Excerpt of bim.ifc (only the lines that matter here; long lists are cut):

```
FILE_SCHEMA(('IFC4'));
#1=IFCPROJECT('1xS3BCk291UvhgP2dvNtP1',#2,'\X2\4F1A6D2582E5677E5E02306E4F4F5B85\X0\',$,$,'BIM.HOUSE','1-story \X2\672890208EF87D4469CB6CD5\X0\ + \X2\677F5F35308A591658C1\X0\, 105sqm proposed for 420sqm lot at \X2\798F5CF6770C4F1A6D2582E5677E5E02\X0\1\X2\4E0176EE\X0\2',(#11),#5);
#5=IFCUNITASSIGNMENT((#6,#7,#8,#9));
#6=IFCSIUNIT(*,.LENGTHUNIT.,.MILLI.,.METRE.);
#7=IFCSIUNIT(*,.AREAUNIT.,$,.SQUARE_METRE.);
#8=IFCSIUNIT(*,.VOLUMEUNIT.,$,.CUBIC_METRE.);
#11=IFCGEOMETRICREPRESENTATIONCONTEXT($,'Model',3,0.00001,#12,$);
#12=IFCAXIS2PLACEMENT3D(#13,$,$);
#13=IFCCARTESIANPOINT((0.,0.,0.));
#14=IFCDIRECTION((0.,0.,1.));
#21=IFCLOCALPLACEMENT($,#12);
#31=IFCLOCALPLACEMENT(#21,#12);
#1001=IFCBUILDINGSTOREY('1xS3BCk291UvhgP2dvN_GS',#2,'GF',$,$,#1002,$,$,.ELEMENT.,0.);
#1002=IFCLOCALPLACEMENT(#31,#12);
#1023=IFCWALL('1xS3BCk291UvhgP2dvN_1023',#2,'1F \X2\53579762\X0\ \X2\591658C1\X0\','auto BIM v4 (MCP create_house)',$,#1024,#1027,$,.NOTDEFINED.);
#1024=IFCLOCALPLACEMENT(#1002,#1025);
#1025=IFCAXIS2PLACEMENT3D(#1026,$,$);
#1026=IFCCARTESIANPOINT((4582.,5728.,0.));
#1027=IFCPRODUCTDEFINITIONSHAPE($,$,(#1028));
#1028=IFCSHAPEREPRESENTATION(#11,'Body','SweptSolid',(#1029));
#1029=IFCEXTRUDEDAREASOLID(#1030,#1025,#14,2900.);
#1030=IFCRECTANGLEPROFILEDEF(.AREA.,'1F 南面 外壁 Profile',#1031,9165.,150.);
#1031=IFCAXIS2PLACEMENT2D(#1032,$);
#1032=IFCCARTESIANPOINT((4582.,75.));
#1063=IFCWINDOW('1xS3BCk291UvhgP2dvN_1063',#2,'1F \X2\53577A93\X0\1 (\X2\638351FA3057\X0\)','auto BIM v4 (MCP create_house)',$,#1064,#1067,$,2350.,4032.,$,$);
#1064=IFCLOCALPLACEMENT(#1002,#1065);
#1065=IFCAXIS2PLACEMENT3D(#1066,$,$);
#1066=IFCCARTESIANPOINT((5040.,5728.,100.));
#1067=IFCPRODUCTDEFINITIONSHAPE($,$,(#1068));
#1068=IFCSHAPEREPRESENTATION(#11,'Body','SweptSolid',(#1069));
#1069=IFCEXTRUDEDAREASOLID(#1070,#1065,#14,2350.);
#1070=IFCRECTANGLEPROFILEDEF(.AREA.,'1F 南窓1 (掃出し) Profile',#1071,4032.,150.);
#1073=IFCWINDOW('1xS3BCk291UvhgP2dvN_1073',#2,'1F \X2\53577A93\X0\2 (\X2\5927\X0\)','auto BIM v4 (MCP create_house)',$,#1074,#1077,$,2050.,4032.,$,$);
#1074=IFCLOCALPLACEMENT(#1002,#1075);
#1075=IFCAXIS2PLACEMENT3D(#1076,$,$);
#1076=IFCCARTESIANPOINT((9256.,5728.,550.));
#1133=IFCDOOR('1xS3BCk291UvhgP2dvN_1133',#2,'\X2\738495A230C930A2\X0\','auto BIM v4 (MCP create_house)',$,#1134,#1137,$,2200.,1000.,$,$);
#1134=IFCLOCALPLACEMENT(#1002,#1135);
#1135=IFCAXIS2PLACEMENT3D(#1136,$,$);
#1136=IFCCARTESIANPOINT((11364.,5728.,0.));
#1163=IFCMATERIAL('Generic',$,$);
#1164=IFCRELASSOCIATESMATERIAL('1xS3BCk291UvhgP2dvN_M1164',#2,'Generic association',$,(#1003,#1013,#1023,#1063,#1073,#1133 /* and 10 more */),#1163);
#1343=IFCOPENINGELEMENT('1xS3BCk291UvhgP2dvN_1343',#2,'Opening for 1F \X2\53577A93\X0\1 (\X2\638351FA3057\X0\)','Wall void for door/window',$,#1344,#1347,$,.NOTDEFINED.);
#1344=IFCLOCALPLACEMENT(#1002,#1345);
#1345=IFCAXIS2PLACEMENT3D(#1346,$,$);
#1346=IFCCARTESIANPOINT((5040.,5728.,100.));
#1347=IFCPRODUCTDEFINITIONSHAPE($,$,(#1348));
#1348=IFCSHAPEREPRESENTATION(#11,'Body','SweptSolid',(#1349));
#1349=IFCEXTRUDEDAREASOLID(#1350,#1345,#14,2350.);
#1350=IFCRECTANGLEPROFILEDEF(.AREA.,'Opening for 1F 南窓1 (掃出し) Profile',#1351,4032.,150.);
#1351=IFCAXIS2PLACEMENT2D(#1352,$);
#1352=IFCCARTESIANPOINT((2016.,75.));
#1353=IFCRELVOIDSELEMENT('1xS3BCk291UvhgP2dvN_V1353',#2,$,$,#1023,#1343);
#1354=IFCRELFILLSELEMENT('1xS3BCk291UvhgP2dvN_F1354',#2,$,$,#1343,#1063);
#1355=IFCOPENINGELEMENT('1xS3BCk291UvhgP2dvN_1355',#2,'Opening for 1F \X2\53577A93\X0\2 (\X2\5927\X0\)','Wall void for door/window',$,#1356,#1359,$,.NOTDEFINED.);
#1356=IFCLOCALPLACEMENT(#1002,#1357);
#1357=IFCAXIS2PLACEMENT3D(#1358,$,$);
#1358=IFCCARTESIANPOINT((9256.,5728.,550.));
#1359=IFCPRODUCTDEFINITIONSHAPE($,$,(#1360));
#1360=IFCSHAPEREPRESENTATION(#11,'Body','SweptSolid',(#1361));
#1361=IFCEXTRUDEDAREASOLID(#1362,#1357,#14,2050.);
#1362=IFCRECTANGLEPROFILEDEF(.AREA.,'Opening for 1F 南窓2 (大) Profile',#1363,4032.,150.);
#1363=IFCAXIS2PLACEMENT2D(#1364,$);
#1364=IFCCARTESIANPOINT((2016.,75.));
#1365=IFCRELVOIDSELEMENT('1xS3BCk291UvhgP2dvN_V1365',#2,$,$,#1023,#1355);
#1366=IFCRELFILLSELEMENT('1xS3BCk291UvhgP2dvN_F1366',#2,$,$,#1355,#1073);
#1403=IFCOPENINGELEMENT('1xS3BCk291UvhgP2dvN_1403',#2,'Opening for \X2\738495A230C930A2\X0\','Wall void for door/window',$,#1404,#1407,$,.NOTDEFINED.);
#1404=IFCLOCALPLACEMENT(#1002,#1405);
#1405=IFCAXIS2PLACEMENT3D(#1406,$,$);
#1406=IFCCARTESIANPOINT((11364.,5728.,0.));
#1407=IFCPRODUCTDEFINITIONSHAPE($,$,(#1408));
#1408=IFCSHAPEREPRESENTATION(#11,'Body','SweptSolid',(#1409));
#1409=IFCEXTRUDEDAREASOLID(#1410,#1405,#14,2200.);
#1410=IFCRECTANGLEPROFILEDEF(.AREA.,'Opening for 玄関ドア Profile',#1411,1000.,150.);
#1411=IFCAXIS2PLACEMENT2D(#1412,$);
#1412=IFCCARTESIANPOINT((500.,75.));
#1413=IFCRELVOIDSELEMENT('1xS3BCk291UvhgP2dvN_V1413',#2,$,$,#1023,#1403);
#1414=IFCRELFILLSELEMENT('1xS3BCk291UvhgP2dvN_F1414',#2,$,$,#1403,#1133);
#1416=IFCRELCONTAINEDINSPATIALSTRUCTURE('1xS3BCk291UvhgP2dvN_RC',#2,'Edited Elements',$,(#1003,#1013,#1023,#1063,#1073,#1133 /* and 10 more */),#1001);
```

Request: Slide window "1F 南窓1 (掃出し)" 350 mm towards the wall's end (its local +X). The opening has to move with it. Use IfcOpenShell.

```python
import ifcopenshell
import ifcopenshell.api.geometry
import ifcopenshell.util.placement
import ifcopenshell.util.unit

model = ifcopenshell.open("bim.ifc")
unit_scale = ifcopenshell.util.unit.calculate_unit_scale(model)

window = model.by_guid("1xS3BCk291UvhgP2dvN_1063")
opening = window.FillsVoids[0].RelatingOpeningElement
wall = opening.VoidsElements[0].RelatingBuildingElement

wall_matrix = ifcopenshell.util.placement.get_local_placement(wall.ObjectPlacement)
shift = wall_matrix[:3, 0] * 0.35 / unit_scale
before = ifcopenshell.util.placement.get_local_placement(window.ObjectPlacement)[:3, 3].copy()

# The window is not placed relative to its opening, so move both.
for product in (opening, window):
    matrix = ifcopenshell.util.placement.get_local_placement(product.ObjectPlacement)
    matrix[:3, 3] += shift
    ifcopenshell.api.geometry.edit_object_placement(model, product=product, matrix=matrix, is_si=False)

after = ifcopenshell.util.placement.get_local_placement(window.ObjectPlacement)[:3, 3]
print("window moved by", (after - before).round(3) + 0.0)

model.write("bim_rev.ifc")
```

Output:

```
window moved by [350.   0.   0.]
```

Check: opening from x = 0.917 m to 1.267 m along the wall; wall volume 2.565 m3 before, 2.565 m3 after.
